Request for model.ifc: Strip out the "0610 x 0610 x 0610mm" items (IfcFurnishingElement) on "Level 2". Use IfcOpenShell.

First a look at what the model holds.

```python
import ifcopenshell
import ifcopenshell.util.element

model = ifcopenshell.open("model.ifc")
print(model.schema)
storey = next(s for s in model.by_type("IfcBuildingStorey") if s.Name == "Level 2")
furniture = [e for e in ifcopenshell.util.element.get_decomposition(storey) if e.is_a("IfcFurnishingElement")]
seen = {}
for e in furniture:
    element_type = ifcopenshell.util.element.get_type(e)
    name = element_type.Name if element_type not in (None, e) else None
    seen[name] = seen.get(name, 0) + 1
for name, count in sorted(seen.items(), key=str):
    print(count, "x", name)
```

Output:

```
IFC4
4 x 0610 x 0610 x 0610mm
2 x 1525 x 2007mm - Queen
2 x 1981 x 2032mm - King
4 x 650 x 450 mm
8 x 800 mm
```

```python
import ifcopenshell
import ifcopenshell.api.root
import ifcopenshell.util.element

model = ifcopenshell.open("model.ifc")

storey = next(s for s in model.by_type("IfcBuildingStorey") if s.Name == "Level 2")
furniture = [e for e in ifcopenshell.util.element.get_decomposition(storey) if e.is_a("IfcFurnishingElement")]
targets = [e for e in furniture if (t := ifcopenshell.util.element.get_type(e)) not in (None, e) and t.Name == "0610 x 0610 x 0610mm"]

for e in targets:
    ifcopenshell.api.root.remove_product(model, product=e)
print(len(targets), "removed")

model.write("model_v2.ifc")
```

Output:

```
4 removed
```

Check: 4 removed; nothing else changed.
